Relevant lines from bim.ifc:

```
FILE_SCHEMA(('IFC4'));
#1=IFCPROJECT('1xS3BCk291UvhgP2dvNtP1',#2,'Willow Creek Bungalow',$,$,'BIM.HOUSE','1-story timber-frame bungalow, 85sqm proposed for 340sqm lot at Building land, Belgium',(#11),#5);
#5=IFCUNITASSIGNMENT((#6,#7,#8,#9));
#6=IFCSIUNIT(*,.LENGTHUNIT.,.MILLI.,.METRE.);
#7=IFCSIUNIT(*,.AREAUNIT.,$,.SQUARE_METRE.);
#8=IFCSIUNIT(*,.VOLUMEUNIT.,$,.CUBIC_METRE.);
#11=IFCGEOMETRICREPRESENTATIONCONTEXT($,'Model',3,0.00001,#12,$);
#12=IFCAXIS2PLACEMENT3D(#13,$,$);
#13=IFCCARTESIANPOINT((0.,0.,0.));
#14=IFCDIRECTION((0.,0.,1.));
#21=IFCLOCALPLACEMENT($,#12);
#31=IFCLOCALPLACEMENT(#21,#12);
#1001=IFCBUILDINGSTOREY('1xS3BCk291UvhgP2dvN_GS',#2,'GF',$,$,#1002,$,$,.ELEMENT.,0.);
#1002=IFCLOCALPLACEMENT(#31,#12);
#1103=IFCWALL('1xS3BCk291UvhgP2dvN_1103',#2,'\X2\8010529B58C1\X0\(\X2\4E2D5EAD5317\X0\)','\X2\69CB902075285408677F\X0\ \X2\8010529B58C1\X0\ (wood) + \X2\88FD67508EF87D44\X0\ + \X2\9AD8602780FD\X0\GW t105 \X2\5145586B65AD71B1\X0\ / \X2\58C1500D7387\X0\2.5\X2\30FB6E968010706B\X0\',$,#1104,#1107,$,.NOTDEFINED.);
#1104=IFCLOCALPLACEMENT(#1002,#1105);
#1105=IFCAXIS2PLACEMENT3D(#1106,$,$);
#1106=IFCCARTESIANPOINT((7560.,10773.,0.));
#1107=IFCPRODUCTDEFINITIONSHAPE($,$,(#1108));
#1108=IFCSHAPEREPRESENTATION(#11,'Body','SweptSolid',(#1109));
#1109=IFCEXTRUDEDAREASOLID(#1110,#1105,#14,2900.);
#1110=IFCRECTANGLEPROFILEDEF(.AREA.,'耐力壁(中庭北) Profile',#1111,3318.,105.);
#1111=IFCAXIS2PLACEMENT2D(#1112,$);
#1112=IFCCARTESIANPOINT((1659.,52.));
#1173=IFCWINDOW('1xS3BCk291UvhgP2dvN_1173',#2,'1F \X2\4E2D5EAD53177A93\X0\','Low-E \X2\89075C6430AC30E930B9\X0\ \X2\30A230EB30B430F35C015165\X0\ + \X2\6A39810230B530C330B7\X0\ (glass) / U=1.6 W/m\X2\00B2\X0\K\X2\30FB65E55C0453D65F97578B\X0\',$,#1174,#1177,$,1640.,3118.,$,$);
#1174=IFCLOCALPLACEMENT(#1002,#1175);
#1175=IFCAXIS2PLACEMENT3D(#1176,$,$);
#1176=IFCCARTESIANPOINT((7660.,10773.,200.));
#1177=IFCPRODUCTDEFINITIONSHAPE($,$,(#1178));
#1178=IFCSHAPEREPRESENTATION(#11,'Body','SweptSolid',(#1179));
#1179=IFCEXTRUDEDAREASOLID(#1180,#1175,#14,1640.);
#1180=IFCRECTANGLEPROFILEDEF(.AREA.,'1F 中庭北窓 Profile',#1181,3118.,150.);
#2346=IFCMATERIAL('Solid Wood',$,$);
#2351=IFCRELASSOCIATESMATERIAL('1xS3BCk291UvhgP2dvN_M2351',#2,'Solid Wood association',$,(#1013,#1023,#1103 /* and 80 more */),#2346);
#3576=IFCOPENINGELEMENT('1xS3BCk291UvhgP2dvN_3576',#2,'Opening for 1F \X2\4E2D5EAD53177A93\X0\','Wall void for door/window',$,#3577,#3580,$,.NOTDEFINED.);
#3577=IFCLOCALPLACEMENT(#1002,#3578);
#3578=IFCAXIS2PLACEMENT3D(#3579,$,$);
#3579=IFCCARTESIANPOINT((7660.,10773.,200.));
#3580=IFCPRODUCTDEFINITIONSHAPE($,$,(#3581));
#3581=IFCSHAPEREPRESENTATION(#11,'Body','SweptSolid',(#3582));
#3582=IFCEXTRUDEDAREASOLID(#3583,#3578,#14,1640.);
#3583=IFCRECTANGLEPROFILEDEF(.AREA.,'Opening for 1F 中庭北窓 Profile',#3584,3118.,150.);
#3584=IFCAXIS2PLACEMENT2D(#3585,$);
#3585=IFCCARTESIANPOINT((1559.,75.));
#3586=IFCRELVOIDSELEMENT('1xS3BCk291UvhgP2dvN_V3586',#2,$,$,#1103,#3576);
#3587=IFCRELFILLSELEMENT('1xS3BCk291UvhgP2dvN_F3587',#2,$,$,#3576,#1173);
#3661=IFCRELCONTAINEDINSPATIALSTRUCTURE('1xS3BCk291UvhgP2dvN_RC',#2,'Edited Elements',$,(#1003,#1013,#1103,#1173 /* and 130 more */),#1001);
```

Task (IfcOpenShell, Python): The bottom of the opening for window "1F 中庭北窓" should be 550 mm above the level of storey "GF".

```python
import numpy as np
import ifcopenshell
import ifcopenshell.api.geometry
import ifcopenshell.geom
import ifcopenshell.util.element
import ifcopenshell.util.placement
import ifcopenshell.util.shape
import ifcopenshell.util.unit

model = ifcopenshell.open("bim.ifc")
unit_scale = ifcopenshell.util.unit.calculate_unit_scale(model)

window = model.by_guid("1xS3BCk291UvhgP2dvN_1173")
opening = window.FillsVoids[0].RelatingOpeningElement
storey = ifcopenshell.util.element.get_container(window, ifc_class="IfcBuildingStorey")
level = ifcopenshell.util.placement.get_local_placement(storey.ObjectPlacement)[2, 3]

# The opening's origin need not be at the sill, so measure its lowest point.
shape = ifcopenshell.geom.create_shape(ifcopenshell.geom.settings(), opening)
bottom = ifcopenshell.util.shape.get_shape_bottom_elevation(shape, shape.geometry) / unit_scale
dz = level + 550.0 - bottom

shift = np.array([0.0, 0.0, dz])
# The window is not placed relative to its opening, so move both.
for product in (opening, window):
    matrix = ifcopenshell.util.placement.get_local_placement(product.ObjectPlacement)
    matrix[:3, 3] += shift
    ifcopenshell.api.geometry.edit_object_placement(model, product=product, matrix=matrix, is_si=False)

print(f"moved by {dz * unit_scale:+.3f} m")

model.write("bim_edited.ifc")
```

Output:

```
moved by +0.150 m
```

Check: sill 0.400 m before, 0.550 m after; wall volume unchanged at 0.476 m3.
